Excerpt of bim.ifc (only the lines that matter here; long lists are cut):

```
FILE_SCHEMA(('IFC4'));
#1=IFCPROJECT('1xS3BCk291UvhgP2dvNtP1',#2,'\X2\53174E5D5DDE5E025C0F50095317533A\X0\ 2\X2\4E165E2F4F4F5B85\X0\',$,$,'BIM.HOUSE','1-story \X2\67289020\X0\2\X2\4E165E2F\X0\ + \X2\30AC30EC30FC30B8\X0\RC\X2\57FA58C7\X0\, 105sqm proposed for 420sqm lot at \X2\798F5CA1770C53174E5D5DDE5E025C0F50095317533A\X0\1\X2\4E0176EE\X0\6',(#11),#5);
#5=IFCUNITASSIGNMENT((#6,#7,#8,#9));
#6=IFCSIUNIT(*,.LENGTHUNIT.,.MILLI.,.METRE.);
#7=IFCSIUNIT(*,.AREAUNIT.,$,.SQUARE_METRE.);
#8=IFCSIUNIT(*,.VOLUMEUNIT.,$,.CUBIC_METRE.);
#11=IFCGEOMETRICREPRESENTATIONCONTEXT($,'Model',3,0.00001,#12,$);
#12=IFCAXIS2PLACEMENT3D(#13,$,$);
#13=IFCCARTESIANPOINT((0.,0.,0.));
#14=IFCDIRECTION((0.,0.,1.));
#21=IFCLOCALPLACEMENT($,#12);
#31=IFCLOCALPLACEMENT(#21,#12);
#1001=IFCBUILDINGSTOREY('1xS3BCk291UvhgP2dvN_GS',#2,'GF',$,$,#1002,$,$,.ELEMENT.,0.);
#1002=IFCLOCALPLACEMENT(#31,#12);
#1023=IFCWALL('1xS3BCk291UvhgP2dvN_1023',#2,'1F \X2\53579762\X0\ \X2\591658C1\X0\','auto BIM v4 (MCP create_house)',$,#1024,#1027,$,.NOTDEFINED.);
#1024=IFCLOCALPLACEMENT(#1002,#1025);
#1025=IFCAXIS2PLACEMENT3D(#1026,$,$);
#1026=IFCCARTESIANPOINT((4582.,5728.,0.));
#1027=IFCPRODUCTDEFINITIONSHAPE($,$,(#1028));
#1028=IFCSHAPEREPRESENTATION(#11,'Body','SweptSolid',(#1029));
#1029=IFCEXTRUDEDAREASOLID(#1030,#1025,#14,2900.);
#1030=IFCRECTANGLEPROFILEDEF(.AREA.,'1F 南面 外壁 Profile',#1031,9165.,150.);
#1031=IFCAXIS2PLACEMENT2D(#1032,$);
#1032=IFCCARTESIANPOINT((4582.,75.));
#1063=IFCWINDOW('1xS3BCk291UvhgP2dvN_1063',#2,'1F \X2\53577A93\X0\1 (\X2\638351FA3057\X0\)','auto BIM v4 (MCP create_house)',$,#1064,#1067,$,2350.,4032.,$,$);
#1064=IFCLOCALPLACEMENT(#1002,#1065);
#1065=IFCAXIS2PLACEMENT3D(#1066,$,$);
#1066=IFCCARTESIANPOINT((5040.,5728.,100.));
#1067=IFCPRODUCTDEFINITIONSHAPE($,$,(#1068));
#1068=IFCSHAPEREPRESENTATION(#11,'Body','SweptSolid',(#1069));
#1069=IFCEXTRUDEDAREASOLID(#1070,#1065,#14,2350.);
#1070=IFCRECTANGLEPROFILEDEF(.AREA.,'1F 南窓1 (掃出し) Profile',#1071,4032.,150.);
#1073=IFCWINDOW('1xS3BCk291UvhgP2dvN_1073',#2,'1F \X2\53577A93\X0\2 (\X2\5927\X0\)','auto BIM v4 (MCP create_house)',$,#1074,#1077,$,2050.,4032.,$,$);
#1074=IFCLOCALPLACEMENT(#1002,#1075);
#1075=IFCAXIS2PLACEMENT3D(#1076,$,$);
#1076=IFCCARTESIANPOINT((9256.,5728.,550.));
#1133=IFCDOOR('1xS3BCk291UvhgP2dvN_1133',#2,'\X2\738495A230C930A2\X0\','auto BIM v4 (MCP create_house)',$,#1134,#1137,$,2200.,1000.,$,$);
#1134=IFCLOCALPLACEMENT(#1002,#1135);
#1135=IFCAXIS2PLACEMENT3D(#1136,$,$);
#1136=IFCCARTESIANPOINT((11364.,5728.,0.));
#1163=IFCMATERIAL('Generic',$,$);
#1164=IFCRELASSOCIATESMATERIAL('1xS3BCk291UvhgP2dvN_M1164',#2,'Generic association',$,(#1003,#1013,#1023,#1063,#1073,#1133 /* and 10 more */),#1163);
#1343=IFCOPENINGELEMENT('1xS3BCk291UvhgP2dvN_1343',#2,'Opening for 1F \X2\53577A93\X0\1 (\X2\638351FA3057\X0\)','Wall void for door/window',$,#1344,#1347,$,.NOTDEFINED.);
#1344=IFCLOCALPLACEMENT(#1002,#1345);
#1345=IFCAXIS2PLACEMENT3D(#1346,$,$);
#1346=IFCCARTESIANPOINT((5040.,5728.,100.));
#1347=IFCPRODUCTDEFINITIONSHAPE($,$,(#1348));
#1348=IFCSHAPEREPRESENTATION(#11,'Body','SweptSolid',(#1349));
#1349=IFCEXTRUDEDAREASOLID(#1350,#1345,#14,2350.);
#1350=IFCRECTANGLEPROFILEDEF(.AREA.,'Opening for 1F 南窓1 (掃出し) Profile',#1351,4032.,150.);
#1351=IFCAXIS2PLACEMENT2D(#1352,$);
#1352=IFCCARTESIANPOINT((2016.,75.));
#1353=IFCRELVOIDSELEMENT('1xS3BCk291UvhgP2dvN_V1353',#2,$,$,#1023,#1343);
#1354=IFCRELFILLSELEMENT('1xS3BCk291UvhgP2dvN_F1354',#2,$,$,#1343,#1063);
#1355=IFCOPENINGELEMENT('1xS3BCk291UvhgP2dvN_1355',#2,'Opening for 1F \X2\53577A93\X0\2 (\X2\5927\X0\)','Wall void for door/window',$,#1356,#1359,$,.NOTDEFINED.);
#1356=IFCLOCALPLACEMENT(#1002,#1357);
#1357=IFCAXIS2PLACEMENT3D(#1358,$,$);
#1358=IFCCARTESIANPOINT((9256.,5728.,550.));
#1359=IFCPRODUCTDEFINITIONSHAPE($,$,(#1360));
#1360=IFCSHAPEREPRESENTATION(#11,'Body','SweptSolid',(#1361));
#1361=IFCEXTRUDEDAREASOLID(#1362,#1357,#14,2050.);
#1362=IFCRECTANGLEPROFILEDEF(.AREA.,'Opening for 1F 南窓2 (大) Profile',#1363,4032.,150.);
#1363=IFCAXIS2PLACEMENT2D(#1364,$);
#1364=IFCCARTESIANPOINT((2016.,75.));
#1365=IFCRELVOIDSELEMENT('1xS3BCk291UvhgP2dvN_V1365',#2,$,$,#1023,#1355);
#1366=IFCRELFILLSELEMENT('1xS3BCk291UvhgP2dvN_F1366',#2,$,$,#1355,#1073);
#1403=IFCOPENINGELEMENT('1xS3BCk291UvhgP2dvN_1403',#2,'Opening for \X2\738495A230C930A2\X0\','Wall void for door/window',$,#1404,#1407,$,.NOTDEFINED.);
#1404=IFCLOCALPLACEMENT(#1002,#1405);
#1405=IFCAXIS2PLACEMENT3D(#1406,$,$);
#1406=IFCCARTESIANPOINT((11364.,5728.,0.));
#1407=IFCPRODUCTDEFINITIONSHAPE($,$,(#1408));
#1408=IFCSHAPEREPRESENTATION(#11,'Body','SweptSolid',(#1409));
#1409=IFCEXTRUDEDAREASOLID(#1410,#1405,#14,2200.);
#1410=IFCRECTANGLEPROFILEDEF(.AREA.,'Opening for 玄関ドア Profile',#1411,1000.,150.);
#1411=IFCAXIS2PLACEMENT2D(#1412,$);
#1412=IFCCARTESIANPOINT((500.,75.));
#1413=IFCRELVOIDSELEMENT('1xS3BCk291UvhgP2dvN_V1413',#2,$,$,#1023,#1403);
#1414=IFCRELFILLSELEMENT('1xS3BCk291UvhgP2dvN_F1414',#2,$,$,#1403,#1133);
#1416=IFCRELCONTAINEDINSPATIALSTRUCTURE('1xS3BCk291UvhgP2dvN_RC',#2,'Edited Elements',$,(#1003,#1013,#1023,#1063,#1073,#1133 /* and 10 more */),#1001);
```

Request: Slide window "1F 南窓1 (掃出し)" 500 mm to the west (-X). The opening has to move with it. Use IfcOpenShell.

```python
import ifcopenshell
import ifcopenshell.api.geometry
import ifcopenshell.util.placement
import ifcopenshell.util.unit

model = ifcopenshell.open("bim.ifc")
unit_scale = ifcopenshell.util.unit.calculate_unit_scale(model)

window = model.by_id(1063)
opening = window.FillsVoids[0].RelatingOpeningElement
wall = opening.VoidsElements[0].RelatingBuildingElement

wall_matrix = ifcopenshell.util.placement.get_local_placement(wall.ObjectPlacement)
shift = wall_matrix[:3, 0] * -0.5 / unit_scale
before = ifcopenshell.util.placement.get_local_placement(window.ObjectPlacement)[:3, 3].copy()

# The window is not placed relative to its opening, so move both.
for product in (opening, window):
    matrix = ifcopenshell.util.placement.get_local_placement(product.ObjectPlacement)
    matrix[:3, 3] += shift
    ifcopenshell.api.geometry.edit_object_placement(model, product=product, matrix=matrix, is_si=False)

after = ifcopenshell.util.placement.get_local_placement(window.ObjectPlacement)[:3, 3]
print("window moved by", (after - before).round(3) + 0.0)

model.write("bim-out.ifc")
```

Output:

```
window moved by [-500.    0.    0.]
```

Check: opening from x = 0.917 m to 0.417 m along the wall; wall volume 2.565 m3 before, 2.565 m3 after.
